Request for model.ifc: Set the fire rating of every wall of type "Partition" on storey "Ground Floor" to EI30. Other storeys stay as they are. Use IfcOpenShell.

First a look at what the model holds.

```python
import ifcopenshell
import ifcopenshell.util.element

model = ifcopenshell.open("model.ifc")
print(model.schema)
storey = next(s for s in model.by_type("IfcBuildingStorey") if s.Name == "Ground Floor")
walls = [e for e in ifcopenshell.util.element.get_decomposition(storey) if e.is_a("IfcWall")]
seen = {}
for e in walls:
    element_type = ifcopenshell.util.element.get_type(e)
    key = (element_type.Name if element_type != e and element_type else None, ifcopenshell.util.element.get_pset(e, "Pset_WallCommon", "FireRating"))
    seen[key] = seen.get(key, 0) + 1
for (name, value), count in sorted(seen.items(), key=str):
    print(count, "x", name, "|", value)
```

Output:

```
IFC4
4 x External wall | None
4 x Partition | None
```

```python
import ifcopenshell
import ifcopenshell.api.pset
import ifcopenshell.util.element

model = ifcopenshell.open("model.ifc")

storey = next(s for s in model.by_type("IfcBuildingStorey") if s.Name == "Ground Floor")
walls = [e for e in ifcopenshell.util.element.get_decomposition(storey) if e.is_a("IfcWall")]

count = 0
for e in walls:
    element_type = ifcopenshell.util.element.get_type(e)
    if element_type in (None, e) or element_type.Name != "Partition":
        continue
    # add_pset returns the element's existing set when there is one.
    pset = ifcopenshell.api.pset.add_pset(model, product=e, name="Pset_WallCommon")
    ifcopenshell.api.pset.edit_pset(model, pset=pset, properties={"FireRating": "EI30"})
    count += 1

print(count, "walls updated")

model.write("model_rev.ifc")
```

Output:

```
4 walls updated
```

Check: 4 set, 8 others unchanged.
